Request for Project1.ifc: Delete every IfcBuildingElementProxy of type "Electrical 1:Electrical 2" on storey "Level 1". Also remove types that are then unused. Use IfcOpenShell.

First a look at what the model holds.

```python
import ifcopenshell
import ifcopenshell.util.element

model = ifcopenshell.open("Project1.ifc")
print(model.schema)
storey = next(s for s in model.by_type("IfcBuildingStorey") if s.Name == "Level 1")
proxies = [e for e in ifcopenshell.util.element.get_decomposition(storey) if e.is_a("IfcBuildingElementProxy")]
seen = {}
for e in proxies:
    element_type = ifcopenshell.util.element.get_type(e)
    name = element_type.Name if element_type not in (None, e) else None
    seen[name] = seen.get(name, 0) + 1
for name, count in sorted(seen.items(), key=str):
    print(count, "x", name)
```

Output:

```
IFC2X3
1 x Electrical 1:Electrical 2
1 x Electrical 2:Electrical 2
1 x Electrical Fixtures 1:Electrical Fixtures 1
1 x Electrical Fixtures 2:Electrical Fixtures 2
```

```python
import ifcopenshell
import ifcopenshell.api.root
import ifcopenshell.util.element

model = ifcopenshell.open("Project1.ifc")

storey = next(s for s in model.by_type("IfcBuildingStorey") if s.Name == "Level 1")
proxies = [e for e in ifcopenshell.util.element.get_decomposition(storey) if e.is_a("IfcBuildingElementProxy")]
targets = [e for e in proxies if (t := ifcopenshell.util.element.get_type(e)) not in (None, e) and t.Name == "Electrical 1:Electrical 2"]
types = {ifcopenshell.util.element.get_type(e) for e in targets} - {None, *targets}

for e in targets:
    ifcopenshell.api.root.remove_product(model, product=e)
print(len(targets), "removed")

unused = [t for t in types if not ifcopenshell.util.element.get_types(t)]
for t in unused:
    ifcopenshell.api.root.remove_product(model, product=t)
print(len(unused), "unused types removed")

model.write("Project1_edited.ifc")
```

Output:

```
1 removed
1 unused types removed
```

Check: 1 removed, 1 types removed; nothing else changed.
